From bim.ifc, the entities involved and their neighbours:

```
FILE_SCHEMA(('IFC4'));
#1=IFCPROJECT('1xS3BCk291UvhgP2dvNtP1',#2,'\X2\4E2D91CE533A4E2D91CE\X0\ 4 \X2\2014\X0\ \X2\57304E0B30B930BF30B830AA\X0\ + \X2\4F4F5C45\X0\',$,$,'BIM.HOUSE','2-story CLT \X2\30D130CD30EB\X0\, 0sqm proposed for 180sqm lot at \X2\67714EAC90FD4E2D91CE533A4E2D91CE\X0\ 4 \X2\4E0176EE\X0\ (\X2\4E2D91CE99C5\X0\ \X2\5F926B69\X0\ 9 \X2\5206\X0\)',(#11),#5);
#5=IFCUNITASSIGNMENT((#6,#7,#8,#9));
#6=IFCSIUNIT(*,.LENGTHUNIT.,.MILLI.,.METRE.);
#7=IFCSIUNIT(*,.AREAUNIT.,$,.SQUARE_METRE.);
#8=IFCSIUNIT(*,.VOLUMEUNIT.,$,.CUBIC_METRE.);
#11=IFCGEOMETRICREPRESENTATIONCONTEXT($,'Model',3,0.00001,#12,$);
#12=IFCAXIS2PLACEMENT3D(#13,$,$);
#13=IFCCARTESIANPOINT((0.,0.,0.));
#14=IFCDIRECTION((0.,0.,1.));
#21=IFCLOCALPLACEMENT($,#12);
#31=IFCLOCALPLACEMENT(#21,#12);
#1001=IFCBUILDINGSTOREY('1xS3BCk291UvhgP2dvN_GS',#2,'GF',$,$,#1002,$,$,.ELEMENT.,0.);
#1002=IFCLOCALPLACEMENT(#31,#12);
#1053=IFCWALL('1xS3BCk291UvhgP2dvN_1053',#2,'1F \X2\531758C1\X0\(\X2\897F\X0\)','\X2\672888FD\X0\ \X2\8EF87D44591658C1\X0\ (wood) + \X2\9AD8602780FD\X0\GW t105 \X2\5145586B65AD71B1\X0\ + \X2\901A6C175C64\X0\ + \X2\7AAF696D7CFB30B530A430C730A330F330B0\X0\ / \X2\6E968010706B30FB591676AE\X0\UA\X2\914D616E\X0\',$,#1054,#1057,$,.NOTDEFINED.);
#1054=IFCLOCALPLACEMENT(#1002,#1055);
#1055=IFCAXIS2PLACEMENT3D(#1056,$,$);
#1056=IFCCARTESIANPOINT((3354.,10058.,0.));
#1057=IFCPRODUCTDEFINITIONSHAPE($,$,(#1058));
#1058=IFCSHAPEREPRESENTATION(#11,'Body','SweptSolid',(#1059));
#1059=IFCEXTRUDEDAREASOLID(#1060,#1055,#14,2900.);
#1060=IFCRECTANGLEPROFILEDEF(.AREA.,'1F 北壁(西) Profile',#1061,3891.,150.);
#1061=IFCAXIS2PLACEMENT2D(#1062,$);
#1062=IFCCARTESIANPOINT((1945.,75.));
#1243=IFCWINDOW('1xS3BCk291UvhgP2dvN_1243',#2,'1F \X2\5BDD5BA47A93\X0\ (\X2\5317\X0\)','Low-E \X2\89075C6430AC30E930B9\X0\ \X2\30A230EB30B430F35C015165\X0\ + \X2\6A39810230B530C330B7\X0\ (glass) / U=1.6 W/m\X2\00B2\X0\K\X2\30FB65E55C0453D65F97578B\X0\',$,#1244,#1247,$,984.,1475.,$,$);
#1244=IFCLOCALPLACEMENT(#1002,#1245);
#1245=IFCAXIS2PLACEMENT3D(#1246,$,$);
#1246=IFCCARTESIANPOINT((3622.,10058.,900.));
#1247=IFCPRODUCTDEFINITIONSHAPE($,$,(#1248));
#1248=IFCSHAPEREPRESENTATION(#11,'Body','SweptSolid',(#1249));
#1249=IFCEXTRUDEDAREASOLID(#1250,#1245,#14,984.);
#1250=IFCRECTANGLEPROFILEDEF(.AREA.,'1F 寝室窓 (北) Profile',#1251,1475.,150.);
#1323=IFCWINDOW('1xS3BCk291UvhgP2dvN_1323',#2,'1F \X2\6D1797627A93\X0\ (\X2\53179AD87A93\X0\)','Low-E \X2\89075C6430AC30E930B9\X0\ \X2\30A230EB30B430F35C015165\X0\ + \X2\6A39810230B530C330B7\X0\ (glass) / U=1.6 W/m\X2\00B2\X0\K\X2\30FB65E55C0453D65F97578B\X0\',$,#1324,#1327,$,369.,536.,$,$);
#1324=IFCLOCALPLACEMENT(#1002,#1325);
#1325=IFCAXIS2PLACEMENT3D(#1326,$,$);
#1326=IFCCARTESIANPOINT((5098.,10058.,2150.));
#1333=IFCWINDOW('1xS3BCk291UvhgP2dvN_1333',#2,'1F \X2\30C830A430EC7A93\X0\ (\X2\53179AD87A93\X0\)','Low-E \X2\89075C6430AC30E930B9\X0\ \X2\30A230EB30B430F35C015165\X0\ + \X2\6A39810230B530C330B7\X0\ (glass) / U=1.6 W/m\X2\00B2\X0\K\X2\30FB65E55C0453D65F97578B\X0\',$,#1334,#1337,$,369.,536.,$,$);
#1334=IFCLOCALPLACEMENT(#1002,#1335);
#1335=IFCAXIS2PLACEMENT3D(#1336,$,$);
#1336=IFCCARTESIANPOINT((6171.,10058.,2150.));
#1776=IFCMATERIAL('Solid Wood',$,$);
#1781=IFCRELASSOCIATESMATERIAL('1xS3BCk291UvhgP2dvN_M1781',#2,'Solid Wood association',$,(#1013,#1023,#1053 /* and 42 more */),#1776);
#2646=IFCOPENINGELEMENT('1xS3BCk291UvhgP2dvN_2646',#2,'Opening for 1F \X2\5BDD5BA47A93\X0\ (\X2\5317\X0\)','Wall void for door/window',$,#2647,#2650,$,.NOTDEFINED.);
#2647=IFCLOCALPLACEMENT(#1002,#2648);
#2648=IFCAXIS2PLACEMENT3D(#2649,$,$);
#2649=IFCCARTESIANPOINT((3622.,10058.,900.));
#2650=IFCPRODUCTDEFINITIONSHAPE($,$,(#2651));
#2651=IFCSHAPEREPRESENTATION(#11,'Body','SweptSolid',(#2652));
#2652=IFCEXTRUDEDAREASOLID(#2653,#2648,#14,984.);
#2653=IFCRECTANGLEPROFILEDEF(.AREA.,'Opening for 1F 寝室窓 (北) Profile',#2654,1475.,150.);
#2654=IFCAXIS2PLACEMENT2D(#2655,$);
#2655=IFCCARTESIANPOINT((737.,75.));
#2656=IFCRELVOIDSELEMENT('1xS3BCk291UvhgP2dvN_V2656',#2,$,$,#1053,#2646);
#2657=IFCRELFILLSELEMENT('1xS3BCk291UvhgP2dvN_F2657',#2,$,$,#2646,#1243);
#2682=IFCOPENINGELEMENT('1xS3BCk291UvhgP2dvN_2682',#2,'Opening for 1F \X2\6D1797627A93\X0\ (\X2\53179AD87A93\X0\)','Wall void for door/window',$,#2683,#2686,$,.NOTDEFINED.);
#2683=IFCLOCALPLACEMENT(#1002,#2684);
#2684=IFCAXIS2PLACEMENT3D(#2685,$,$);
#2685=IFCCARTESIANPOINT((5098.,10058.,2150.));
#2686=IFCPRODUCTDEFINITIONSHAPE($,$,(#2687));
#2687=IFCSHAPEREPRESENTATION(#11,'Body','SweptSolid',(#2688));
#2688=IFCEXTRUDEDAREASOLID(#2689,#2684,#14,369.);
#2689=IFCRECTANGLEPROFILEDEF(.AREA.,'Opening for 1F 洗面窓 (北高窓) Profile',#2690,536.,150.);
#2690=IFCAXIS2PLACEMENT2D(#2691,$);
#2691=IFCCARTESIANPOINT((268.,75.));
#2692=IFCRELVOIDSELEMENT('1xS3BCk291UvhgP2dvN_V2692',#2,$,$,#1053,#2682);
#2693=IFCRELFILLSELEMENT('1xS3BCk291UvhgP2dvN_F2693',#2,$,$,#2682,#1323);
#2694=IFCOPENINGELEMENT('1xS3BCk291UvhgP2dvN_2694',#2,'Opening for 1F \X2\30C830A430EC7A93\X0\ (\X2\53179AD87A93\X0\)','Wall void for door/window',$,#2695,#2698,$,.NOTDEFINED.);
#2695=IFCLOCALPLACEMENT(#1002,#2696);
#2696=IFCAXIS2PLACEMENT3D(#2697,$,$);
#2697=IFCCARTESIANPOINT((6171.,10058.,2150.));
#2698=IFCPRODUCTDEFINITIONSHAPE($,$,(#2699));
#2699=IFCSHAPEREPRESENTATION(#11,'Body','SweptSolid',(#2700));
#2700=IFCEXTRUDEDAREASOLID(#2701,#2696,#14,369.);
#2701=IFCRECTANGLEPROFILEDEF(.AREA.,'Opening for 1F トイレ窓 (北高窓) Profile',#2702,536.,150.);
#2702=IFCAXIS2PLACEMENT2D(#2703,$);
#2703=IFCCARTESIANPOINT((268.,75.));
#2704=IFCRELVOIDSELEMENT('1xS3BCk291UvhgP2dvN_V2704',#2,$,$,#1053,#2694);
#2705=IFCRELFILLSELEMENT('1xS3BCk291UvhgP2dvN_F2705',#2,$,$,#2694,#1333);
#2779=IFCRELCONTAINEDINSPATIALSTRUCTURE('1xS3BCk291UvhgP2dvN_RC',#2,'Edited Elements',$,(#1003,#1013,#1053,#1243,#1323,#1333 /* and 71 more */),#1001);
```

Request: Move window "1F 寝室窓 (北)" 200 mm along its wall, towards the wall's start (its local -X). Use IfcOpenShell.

```python
import ifcopenshell
import ifcopenshell.api.geometry
import ifcopenshell.util.placement
import ifcopenshell.util.unit

model = ifcopenshell.open("bim.ifc")
unit_scale = ifcopenshell.util.unit.calculate_unit_scale(model)

window = model.by_guid("1xS3BCk291UvhgP2dvN_1243")
opening = window.FillsVoids[0].RelatingOpeningElement
wall = opening.VoidsElements[0].RelatingBuildingElement

wall_matrix = ifcopenshell.util.placement.get_local_placement(wall.ObjectPlacement)
shift = wall_matrix[:3, 0] * -0.2 / unit_scale
before = ifcopenshell.util.placement.get_local_placement(window.ObjectPlacement)[:3, 3].copy()

# The window is not placed relative to its opening, so move both.
for product in (opening, window):
    matrix = ifcopenshell.util.placement.get_local_placement(product.ObjectPlacement)
    matrix[:3, 3] += shift
    ifcopenshell.api.geometry.edit_object_placement(model, product=product, matrix=matrix, is_si=False)

after = ifcopenshell.util.placement.get_local_placement(window.ObjectPlacement)[:3, 3]
print("window moved by", (after - before).round(3) + 0.0)

model.write("bim_rev.ifc")
```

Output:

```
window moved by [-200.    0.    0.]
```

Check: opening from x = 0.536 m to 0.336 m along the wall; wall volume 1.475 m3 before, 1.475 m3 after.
